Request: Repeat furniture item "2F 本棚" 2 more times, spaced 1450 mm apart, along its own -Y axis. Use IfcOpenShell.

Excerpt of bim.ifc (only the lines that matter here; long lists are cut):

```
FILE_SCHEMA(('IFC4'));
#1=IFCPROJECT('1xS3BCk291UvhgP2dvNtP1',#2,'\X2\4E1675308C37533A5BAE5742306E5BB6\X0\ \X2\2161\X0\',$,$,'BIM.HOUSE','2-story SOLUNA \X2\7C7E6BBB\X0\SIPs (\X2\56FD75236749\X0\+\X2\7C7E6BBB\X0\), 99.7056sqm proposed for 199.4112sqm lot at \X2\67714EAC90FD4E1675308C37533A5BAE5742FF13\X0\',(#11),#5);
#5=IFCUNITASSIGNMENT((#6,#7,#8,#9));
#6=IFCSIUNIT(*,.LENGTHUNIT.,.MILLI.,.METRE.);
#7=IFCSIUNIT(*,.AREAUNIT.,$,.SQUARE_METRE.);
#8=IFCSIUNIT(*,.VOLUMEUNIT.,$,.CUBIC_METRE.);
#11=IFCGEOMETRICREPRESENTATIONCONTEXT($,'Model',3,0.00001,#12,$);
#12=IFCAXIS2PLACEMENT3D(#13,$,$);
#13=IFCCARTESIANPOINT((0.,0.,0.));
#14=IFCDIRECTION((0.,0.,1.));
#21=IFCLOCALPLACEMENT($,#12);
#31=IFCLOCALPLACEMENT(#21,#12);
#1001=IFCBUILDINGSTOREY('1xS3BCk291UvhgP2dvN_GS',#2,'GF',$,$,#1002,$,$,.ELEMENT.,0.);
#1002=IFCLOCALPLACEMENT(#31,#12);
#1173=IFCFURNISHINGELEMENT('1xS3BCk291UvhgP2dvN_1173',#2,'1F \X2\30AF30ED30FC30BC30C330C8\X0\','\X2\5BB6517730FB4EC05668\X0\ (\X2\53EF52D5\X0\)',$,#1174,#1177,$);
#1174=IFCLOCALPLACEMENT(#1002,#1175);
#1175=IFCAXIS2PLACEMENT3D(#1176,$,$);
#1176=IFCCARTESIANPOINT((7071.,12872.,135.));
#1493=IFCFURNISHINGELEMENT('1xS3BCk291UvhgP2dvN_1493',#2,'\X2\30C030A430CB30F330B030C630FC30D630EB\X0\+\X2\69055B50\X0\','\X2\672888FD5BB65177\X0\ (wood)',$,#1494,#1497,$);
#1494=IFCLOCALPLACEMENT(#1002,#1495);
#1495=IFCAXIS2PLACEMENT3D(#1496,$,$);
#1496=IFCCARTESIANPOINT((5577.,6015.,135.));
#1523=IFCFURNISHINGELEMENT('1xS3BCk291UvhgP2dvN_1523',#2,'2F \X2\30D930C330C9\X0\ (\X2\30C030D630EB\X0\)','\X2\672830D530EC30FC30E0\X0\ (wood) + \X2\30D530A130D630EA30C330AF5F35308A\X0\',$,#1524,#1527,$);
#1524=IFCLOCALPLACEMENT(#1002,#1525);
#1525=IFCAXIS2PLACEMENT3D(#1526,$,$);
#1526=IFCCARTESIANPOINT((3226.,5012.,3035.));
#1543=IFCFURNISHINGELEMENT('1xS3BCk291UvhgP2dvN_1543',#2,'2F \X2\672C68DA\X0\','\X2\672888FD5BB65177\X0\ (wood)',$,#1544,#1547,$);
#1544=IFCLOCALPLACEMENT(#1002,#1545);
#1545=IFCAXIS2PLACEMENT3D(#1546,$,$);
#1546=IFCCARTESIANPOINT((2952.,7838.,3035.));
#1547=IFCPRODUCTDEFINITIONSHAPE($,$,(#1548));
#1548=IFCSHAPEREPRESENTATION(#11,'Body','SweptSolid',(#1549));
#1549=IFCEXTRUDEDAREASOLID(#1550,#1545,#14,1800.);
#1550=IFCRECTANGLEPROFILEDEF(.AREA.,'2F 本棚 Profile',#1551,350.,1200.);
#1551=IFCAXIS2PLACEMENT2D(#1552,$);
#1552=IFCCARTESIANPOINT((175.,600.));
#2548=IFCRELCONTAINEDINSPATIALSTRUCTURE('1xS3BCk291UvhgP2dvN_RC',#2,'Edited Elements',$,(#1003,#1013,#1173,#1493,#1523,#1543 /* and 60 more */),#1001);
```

```python
import ifcopenshell
import ifcopenshell.api.geometry
import ifcopenshell.api.root
import ifcopenshell.util.element
import ifcopenshell.util.placement

model = ifcopenshell.open("bim.ifc")


def reuse_history(source, copy):
    """copy_class also copies each property set's owner history, people and application; keep the originals."""
    for rel in copy.IsDefinedBy:
        if rel.is_a("IfcRelDefinesByProperties") and (history := rel.RelatingPropertyDefinition.OwnerHistory):
            rel.RelatingPropertyDefinition.OwnerHistory = source.OwnerHistory
            ifcopenshell.util.element.remove_deep2(model, history)


source = model.by_id(1543)
base = ifcopenshell.util.placement.get_local_placement(source.ObjectPlacement)
step = -base[:3, 1] * 1450.0

for i in range(1, 3):
    copy = ifcopenshell.api.root.copy_class(model, product=source)
    copy.Representation = ifcopenshell.util.element.copy_deep(
        model, source.Representation, exclude=["IfcGeometricRepresentationContext", "IfcRepresentationMap"]
    )
    reuse_history(source, copy)
    matrix = base.copy()
    matrix[:3, 3] += i * step
    print("added at", matrix[:3, 3].round(3) + 0.0)
    ifcopenshell.api.geometry.edit_object_placement(model, product=copy, matrix=matrix, is_si=False)

model.write("bim-out.ifc")
```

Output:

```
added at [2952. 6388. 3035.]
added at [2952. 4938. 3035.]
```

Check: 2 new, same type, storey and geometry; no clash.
